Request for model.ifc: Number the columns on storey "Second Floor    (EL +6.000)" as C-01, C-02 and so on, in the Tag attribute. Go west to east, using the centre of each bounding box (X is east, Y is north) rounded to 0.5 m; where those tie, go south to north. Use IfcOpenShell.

First a look at what the model holds.

```python
import ifcopenshell
import ifcopenshell.util.element
import ifcopenshell.util.placement

model = ifcopenshell.open("model.ifc")
print(model.schema)
storey = next(s for s in model.by_type("IfcBuildingStorey") if s.Name == "Second Floor    (EL +6.000)")
columns = [e for e in ifcopenshell.util.element.get_decomposition(storey) if e.is_a("IfcColumn")]
for e in sorted(columns, key=lambda e: e.id()):
    origin = ifcopenshell.util.placement.get_local_placement(e.ObjectPlacement)[:3, 3]
    print(e.id(), e.Tag, e.Name, origin.round(2) + 0.0, sep=" | ")
```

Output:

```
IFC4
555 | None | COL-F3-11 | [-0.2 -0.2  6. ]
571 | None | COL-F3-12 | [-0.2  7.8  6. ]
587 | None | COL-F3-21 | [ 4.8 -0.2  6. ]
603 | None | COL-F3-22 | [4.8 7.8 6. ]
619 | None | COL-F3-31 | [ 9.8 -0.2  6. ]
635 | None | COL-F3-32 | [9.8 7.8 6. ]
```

```python
import ifcopenshell
import ifcopenshell.geom
import ifcopenshell.util.element
import ifcopenshell.util.shape

model = ifcopenshell.open("model.ifc")
settings = ifcopenshell.geom.settings()
settings.set("use-world-coords", True)


def centre(element):
    shape = ifcopenshell.geom.create_shape(settings, element)
    return ifcopenshell.util.shape.get_bbox_centroid(shape.geometry)


storey = next(s for s in model.by_type("IfcBuildingStorey") if s.Name == "Second Floor    (EL +6.000)")
columns = [e for e in ifcopenshell.util.element.get_decomposition(storey) if e.is_a("IfcColumn")]

# Insertion points can sit at a corner or the storey origin, so sort by the geometry (in metres).
centres = {e: centre(e) for e in columns}
columns.sort(key=lambda e: (round(centres[e][0] / 0.5), centres[e][1]))

for i, e in enumerate(columns, start=1):
    number = f"C-{i:02d}"
    e.Tag = number
    print(e.id(), number)

model.write("model_rev.ifc")
```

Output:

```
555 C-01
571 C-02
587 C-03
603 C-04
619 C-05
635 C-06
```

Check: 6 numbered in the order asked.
